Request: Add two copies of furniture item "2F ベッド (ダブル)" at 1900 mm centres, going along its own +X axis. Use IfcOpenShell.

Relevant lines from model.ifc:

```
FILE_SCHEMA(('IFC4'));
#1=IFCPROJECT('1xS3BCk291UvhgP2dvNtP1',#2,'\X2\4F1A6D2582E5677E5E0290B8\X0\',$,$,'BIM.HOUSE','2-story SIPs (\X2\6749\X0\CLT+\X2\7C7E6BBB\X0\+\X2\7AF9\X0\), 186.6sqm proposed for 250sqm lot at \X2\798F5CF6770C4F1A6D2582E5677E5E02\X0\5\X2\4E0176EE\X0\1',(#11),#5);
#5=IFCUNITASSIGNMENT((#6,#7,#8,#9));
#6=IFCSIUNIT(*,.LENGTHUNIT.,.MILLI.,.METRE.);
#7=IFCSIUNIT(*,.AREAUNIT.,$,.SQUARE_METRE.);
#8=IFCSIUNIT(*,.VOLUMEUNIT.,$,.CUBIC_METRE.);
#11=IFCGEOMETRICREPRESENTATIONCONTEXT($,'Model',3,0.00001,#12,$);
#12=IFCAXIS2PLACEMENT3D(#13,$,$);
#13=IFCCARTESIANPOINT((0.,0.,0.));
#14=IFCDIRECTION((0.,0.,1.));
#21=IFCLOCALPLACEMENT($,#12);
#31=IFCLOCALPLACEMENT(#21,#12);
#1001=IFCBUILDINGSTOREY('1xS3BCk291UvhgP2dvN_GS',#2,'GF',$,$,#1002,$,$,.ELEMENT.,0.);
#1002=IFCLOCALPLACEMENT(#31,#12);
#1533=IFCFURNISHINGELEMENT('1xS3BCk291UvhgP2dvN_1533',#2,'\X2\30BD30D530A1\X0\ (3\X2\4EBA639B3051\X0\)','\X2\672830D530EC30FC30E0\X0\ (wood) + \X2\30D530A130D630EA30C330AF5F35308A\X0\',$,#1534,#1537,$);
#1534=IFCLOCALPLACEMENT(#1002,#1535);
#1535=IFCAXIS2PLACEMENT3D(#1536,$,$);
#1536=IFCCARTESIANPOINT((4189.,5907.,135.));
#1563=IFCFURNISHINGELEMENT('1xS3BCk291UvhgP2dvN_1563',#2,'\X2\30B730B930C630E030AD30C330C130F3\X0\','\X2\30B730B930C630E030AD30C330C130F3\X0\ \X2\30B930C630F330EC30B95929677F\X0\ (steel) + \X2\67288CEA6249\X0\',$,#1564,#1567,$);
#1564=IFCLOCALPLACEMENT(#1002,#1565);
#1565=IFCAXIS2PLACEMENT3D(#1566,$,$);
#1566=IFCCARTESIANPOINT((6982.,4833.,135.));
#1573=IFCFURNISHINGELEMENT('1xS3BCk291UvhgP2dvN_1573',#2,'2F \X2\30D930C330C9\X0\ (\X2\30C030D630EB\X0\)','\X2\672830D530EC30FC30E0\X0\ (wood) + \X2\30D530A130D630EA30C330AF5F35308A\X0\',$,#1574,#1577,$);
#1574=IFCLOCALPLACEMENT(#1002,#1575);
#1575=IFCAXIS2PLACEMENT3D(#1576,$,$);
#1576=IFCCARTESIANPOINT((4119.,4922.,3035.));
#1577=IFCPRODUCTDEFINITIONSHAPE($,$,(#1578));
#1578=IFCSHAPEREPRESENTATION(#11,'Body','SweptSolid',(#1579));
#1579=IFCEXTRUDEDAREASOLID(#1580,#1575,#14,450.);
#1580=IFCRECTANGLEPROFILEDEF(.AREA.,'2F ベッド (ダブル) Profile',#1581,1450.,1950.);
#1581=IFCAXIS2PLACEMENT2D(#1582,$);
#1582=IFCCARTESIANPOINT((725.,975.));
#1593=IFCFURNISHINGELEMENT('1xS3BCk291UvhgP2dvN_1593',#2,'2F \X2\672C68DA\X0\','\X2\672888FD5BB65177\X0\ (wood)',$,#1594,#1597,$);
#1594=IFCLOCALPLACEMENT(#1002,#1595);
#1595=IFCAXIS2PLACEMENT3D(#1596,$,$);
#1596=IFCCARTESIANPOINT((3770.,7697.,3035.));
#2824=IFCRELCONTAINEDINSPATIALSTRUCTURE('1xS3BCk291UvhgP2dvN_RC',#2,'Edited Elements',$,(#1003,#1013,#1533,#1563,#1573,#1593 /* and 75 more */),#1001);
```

```python
import ifcopenshell
import ifcopenshell.api.geometry
import ifcopenshell.api.root
import ifcopenshell.util.element
import ifcopenshell.util.placement
import ifcopenshell.util.unit

model = ifcopenshell.open("model.ifc")
unit_scale = ifcopenshell.util.unit.calculate_unit_scale(model)


def reuse_history(source, copy):
    """copy_class also copies each property set's owner history, people and application; keep the originals."""
    for rel in copy.IsDefinedBy:
        if rel.is_a("IfcRelDefinesByProperties") and (history := rel.RelatingPropertyDefinition.OwnerHistory):
            rel.RelatingPropertyDefinition.OwnerHistory = source.OwnerHistory
            ifcopenshell.util.element.remove_deep2(model, history)


source = model.by_id(1573)
base = ifcopenshell.util.placement.get_local_placement(source.ObjectPlacement)
step = base[:3, 0] * 1.9 / unit_scale

for i in range(1, 3):
    copy = ifcopenshell.api.root.copy_class(model, product=source)
    copy.Representation = ifcopenshell.util.element.copy_deep(
        model, source.Representation, exclude=["IfcGeometricRepresentationContext", "IfcRepresentationMap"]
    )
    reuse_history(source, copy)
    matrix = base.copy()
    matrix[:3, 3] += i * step
    print("added at", matrix[:3, 3].round(3) + 0.0)
    ifcopenshell.api.geometry.edit_object_placement(model, product=copy, matrix=matrix, is_si=False)

model.write("model-out.ifc")
```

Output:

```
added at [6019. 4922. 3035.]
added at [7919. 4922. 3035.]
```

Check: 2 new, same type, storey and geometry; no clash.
